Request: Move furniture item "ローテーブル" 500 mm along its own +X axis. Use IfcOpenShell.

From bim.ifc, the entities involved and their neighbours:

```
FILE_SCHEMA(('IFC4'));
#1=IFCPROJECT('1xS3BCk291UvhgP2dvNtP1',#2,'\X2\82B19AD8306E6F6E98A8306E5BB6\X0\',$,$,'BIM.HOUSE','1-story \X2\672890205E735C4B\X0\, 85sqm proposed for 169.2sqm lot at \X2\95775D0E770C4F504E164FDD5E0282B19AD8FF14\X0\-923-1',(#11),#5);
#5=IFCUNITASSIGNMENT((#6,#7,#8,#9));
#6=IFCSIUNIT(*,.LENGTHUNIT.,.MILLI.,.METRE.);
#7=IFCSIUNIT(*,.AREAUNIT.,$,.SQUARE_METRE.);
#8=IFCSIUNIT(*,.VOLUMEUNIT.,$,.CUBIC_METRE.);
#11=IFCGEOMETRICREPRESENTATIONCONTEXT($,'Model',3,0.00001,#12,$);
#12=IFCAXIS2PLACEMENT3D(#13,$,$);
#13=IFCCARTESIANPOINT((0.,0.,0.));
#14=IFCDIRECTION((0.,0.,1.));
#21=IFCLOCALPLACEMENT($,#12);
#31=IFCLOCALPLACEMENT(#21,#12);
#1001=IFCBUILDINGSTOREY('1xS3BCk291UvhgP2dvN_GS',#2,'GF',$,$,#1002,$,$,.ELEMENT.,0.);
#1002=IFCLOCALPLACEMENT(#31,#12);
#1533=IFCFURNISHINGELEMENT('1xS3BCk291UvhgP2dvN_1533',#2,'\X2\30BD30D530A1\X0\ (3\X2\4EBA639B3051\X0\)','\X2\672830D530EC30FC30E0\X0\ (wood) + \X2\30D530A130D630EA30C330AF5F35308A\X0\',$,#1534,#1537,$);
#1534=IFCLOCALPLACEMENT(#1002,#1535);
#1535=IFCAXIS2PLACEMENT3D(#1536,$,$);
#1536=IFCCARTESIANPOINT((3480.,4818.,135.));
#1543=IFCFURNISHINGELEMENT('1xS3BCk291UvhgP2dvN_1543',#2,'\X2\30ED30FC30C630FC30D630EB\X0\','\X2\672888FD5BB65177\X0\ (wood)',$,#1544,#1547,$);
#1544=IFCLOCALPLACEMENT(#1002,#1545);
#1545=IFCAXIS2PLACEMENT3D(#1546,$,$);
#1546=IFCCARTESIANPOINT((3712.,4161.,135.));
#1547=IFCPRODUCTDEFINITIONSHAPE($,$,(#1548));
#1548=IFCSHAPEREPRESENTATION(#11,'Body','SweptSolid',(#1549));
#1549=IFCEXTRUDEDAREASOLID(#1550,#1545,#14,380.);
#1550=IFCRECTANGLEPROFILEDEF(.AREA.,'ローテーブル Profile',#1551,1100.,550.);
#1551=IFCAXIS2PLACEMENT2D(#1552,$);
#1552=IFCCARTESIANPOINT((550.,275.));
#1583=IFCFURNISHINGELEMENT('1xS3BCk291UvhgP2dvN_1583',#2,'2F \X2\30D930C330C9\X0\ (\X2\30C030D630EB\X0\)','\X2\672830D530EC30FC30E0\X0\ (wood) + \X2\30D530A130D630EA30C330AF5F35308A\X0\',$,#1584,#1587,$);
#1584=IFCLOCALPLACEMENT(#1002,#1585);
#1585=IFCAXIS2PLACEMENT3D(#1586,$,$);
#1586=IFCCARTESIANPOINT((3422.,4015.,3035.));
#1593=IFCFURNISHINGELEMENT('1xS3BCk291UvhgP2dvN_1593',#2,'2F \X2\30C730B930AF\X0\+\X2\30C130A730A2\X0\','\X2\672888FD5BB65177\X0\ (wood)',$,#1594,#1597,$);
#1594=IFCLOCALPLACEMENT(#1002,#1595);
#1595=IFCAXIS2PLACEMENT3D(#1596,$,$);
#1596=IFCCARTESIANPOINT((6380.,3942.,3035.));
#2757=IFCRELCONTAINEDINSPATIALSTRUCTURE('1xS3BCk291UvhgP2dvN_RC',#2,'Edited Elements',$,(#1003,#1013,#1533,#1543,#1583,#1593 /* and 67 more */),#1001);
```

```python
import ifcopenshell
import ifcopenshell.api.geometry
import ifcopenshell.util.placement

model = ifcopenshell.open("bim.ifc")

item = model.by_guid("1xS3BCk291UvhgP2dvN_1543")
matrix = ifcopenshell.util.placement.get_local_placement(item.ObjectPlacement)
matrix[:3, 3] += matrix[:3, 0] * 500.0
ifcopenshell.api.geometry.edit_object_placement(model, product=item, matrix=matrix, is_si=False)

print(ifcopenshell.util.placement.get_local_placement(item.ObjectPlacement).round(3) + 0.0)

model.write("bim_edited.ifc")
```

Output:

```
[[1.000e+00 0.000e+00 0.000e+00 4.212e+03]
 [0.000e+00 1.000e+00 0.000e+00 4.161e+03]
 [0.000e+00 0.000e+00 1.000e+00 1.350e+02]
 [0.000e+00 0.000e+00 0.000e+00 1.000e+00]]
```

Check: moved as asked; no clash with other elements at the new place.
